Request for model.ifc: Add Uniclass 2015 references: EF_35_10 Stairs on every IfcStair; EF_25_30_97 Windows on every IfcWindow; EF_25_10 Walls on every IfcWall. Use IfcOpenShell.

First a look at what the model holds.

```python
import ifcopenshell

model = ifcopenshell.open("model.ifc")
print(model.schema)
print("classifications:", [c.Name for c in model.by_type("IfcClassification")])
for ifc_class in ("IfcDoor", "IfcRoof", "IfcStair", "IfcWall", "IfcWindow"):
    print(ifc_class, len(model.by_type(ifc_class)))
```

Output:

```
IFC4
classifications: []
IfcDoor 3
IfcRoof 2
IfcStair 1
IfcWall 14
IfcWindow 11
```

```python
import ifcopenshell
import ifcopenshell.api.classification

model = ifcopenshell.open("model.ifc")

system = ifcopenshell.api.classification.add_classification(model, classification="Uniclass 2015")

codes = {
    "IfcStair": ("EF_35_10", "Stairs"),
    "IfcWindow": ("EF_25_30_97", "Windows"),
    "IfcWall": ("EF_25_10", "Walls"),
}
for ifc_class, (code, name) in codes.items():
    products = model.by_type(ifc_class)
    ifcopenshell.api.classification.add_reference(
        model, products=products, classification=system, identification=code, name=name
    )
    print(code, len(products))

model.write("model_updated.ifc")
```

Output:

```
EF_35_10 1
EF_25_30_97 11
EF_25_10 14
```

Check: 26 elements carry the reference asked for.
